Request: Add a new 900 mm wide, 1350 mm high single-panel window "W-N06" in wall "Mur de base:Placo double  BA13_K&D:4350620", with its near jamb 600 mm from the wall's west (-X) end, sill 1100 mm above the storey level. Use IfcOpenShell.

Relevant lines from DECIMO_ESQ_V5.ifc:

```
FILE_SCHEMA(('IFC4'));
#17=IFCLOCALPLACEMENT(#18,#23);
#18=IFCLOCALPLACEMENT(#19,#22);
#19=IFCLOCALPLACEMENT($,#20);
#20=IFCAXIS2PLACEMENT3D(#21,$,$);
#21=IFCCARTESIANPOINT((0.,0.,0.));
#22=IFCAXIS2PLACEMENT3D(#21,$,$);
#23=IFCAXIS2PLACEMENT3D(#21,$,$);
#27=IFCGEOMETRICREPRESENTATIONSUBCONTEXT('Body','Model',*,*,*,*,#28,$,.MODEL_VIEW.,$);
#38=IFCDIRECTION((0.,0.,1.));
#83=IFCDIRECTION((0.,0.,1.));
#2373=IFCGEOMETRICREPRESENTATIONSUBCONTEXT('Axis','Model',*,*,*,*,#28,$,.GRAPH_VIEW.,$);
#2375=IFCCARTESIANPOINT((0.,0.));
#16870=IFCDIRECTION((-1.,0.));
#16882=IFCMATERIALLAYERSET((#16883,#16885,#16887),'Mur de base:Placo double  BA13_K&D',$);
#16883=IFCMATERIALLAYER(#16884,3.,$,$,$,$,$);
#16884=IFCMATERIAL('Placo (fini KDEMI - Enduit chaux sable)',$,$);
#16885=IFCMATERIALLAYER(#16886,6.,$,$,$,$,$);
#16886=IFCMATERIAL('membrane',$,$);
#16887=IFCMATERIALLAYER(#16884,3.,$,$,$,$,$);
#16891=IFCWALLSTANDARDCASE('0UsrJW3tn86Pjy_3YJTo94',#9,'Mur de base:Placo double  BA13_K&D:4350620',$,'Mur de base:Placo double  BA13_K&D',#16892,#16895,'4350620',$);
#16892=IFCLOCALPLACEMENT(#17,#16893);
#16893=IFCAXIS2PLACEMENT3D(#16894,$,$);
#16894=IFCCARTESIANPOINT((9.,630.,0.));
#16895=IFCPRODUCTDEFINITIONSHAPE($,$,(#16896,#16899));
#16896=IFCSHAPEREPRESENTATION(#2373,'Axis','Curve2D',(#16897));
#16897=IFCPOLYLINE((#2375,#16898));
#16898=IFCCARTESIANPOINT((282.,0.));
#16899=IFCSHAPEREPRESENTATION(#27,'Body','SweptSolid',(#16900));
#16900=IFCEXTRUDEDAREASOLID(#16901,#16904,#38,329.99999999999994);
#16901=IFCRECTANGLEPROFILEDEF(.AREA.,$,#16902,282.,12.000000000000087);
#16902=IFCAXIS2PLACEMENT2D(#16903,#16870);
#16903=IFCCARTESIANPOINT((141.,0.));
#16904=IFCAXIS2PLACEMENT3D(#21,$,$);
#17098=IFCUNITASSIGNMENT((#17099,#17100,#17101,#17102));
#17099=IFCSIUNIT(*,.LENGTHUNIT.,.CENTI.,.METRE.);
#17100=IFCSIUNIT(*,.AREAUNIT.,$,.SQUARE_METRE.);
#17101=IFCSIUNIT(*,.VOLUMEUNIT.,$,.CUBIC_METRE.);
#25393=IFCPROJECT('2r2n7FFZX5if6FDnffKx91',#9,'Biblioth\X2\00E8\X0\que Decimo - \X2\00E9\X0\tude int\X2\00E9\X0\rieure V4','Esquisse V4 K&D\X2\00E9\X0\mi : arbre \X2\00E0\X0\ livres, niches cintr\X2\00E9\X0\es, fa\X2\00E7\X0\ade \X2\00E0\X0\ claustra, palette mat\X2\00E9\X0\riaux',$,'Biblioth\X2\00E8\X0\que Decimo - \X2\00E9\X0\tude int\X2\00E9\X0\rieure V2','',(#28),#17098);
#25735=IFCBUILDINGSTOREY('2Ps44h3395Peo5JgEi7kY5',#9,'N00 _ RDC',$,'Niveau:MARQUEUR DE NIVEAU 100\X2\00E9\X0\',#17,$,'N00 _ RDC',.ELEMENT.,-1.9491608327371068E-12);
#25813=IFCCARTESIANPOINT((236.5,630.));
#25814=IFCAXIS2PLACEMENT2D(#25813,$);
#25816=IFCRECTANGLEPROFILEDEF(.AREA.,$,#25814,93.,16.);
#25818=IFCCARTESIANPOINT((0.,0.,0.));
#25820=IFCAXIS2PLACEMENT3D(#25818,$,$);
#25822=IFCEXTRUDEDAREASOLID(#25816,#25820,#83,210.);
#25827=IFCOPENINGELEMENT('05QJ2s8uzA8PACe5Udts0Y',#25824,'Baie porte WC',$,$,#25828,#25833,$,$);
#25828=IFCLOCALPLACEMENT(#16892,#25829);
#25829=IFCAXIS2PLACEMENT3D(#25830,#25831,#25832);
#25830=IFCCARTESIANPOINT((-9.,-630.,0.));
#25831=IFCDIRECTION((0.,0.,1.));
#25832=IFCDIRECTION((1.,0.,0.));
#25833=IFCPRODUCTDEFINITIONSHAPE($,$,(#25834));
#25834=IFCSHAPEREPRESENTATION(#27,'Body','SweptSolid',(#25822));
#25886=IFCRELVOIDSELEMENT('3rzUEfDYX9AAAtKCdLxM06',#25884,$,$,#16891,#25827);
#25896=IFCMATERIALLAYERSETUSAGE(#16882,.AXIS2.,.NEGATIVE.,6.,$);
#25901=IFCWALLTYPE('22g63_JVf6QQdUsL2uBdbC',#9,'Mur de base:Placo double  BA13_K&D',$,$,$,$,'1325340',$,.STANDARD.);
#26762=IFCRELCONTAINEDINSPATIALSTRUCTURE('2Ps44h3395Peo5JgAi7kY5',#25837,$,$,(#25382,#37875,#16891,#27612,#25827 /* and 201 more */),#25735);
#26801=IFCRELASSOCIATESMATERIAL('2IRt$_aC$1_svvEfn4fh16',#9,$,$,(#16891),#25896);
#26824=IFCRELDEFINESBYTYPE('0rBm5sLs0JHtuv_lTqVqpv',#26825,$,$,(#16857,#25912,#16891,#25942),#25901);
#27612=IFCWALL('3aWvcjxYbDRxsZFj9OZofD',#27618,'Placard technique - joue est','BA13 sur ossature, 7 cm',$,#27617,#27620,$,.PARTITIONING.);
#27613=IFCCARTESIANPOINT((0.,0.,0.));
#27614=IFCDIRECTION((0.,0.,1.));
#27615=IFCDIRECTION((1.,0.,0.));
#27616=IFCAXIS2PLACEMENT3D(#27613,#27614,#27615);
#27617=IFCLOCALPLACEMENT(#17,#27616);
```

```python
import numpy as np
import ifcopenshell
import ifcopenshell.api.feature
import ifcopenshell.api.geometry
import ifcopenshell.api.root
import ifcopenshell.api.spatial
import ifcopenshell.geom
import ifcopenshell.util.element
import ifcopenshell.util.placement
import ifcopenshell.util.representation
import ifcopenshell.util.shape
import ifcopenshell.util.unit

model = ifcopenshell.open("DECIMO_ESQ_V5.ifc")
unit_scale = ifcopenshell.util.unit.calculate_unit_scale(model)
settings = ifcopenshell.geom.settings()


def volume(element):
    """Net volume in cubic metres, openings subtracted."""
    shape = ifcopenshell.geom.create_shape(settings, element)
    return ifcopenshell.util.shape.get_volume(shape.geometry)


wall = model.by_guid("0UsrJW3tn86Pjy_3YJTo94")
storey = ifcopenshell.util.element.get_container(wall, ifc_class="IfcBuildingStorey")
context = ifcopenshell.util.representation.get_context(model, "Model", "Body", "MODEL_VIEW")
before = volume(wall)

width, height, from_end, sill = 0.9, 1.35, 0.6, 1.1  # metres

# The wall runs along its own X axis, and the end named is its -X end.
wall_shape = ifcopenshell.geom.create_shape(settings, wall)
x, y, z = ifcopenshell.util.shape.get_vertices(wall_shape.geometry).T
start = x.min() + from_end
face, thickness = float(y.min()), float(y.max() - y.min())
wall_matrix = ifcopenshell.util.placement.get_local_placement(wall.ObjectPlacement)
level = ifcopenshell.util.placement.get_local_placement(storey.ObjectPlacement)[2, 3]


def in_wall(x, y):
    """Placement at x, y metres in the wall's axes, at sill height."""
    matrix = wall_matrix.copy()
    matrix[:, 3] = wall_matrix @ np.array([x / unit_scale, y / unit_scale, 0.0, 1.0])
    matrix[2, 3] = level + sill / unit_scale
    return matrix


# Opening: a box that overshoots both wall faces by 50 mm.
opening = ifcopenshell.api.root.create_entity(model, ifc_class="IfcOpeningElement", predefined_type="OPENING")
box = ifcopenshell.api.geometry.add_wall_representation(
    model, context=context, length=width, height=height, thickness=thickness + 0.1
)
ifcopenshell.api.geometry.assign_representation(model, product=opening, representation=box)
ifcopenshell.api.geometry.edit_object_placement(model, product=opening, matrix=in_wall(start, face - 0.05), is_si=False)
ifcopenshell.api.feature.add_feature(model, feature=opening, element=wall)

window = ifcopenshell.api.root.create_entity(model, ifc_class="IfcWindow", name="W-N06", predefined_type="WINDOW")
window.OverallWidth, window.OverallHeight = width / unit_scale, height / unit_scale
window.PartitioningType = "SINGLE_PANEL"
body = ifcopenshell.api.geometry.add_window_representation(
    model,
    context=context,
    overall_width=window.OverallWidth,
    overall_height=window.OverallHeight,
    partition_type="SINGLE_PANEL",
)
ifcopenshell.api.geometry.assign_representation(model, product=window, representation=body)
ifcopenshell.api.spatial.assign_container(model, products=[window], relating_structure=storey)
ifcopenshell.api.feature.add_filling(model, opening=opening, element=window)

# Centre the window in the wall's thickness.
ifcopenshell.api.geometry.edit_object_placement(model, product=window, matrix=in_wall(start, face), is_si=False)
window_shape = ifcopenshell.geom.create_shape(settings, window)
depth = ifcopenshell.util.shape.get_vertices(window_shape.geometry)[:, 1]
offset = face + thickness / 2 - (depth.min() + depth.max()) / 2
ifcopenshell.api.geometry.edit_object_placement(model, product=window, matrix=in_wall(start, offset), is_si=False)

after = volume(wall)

print(f"wall volume {before:.3f} -> {after:.3f} m3")

model.write("DECIMO_ESQ_V5_v2.ifc")
```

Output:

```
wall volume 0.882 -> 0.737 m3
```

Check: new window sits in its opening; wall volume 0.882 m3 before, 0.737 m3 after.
